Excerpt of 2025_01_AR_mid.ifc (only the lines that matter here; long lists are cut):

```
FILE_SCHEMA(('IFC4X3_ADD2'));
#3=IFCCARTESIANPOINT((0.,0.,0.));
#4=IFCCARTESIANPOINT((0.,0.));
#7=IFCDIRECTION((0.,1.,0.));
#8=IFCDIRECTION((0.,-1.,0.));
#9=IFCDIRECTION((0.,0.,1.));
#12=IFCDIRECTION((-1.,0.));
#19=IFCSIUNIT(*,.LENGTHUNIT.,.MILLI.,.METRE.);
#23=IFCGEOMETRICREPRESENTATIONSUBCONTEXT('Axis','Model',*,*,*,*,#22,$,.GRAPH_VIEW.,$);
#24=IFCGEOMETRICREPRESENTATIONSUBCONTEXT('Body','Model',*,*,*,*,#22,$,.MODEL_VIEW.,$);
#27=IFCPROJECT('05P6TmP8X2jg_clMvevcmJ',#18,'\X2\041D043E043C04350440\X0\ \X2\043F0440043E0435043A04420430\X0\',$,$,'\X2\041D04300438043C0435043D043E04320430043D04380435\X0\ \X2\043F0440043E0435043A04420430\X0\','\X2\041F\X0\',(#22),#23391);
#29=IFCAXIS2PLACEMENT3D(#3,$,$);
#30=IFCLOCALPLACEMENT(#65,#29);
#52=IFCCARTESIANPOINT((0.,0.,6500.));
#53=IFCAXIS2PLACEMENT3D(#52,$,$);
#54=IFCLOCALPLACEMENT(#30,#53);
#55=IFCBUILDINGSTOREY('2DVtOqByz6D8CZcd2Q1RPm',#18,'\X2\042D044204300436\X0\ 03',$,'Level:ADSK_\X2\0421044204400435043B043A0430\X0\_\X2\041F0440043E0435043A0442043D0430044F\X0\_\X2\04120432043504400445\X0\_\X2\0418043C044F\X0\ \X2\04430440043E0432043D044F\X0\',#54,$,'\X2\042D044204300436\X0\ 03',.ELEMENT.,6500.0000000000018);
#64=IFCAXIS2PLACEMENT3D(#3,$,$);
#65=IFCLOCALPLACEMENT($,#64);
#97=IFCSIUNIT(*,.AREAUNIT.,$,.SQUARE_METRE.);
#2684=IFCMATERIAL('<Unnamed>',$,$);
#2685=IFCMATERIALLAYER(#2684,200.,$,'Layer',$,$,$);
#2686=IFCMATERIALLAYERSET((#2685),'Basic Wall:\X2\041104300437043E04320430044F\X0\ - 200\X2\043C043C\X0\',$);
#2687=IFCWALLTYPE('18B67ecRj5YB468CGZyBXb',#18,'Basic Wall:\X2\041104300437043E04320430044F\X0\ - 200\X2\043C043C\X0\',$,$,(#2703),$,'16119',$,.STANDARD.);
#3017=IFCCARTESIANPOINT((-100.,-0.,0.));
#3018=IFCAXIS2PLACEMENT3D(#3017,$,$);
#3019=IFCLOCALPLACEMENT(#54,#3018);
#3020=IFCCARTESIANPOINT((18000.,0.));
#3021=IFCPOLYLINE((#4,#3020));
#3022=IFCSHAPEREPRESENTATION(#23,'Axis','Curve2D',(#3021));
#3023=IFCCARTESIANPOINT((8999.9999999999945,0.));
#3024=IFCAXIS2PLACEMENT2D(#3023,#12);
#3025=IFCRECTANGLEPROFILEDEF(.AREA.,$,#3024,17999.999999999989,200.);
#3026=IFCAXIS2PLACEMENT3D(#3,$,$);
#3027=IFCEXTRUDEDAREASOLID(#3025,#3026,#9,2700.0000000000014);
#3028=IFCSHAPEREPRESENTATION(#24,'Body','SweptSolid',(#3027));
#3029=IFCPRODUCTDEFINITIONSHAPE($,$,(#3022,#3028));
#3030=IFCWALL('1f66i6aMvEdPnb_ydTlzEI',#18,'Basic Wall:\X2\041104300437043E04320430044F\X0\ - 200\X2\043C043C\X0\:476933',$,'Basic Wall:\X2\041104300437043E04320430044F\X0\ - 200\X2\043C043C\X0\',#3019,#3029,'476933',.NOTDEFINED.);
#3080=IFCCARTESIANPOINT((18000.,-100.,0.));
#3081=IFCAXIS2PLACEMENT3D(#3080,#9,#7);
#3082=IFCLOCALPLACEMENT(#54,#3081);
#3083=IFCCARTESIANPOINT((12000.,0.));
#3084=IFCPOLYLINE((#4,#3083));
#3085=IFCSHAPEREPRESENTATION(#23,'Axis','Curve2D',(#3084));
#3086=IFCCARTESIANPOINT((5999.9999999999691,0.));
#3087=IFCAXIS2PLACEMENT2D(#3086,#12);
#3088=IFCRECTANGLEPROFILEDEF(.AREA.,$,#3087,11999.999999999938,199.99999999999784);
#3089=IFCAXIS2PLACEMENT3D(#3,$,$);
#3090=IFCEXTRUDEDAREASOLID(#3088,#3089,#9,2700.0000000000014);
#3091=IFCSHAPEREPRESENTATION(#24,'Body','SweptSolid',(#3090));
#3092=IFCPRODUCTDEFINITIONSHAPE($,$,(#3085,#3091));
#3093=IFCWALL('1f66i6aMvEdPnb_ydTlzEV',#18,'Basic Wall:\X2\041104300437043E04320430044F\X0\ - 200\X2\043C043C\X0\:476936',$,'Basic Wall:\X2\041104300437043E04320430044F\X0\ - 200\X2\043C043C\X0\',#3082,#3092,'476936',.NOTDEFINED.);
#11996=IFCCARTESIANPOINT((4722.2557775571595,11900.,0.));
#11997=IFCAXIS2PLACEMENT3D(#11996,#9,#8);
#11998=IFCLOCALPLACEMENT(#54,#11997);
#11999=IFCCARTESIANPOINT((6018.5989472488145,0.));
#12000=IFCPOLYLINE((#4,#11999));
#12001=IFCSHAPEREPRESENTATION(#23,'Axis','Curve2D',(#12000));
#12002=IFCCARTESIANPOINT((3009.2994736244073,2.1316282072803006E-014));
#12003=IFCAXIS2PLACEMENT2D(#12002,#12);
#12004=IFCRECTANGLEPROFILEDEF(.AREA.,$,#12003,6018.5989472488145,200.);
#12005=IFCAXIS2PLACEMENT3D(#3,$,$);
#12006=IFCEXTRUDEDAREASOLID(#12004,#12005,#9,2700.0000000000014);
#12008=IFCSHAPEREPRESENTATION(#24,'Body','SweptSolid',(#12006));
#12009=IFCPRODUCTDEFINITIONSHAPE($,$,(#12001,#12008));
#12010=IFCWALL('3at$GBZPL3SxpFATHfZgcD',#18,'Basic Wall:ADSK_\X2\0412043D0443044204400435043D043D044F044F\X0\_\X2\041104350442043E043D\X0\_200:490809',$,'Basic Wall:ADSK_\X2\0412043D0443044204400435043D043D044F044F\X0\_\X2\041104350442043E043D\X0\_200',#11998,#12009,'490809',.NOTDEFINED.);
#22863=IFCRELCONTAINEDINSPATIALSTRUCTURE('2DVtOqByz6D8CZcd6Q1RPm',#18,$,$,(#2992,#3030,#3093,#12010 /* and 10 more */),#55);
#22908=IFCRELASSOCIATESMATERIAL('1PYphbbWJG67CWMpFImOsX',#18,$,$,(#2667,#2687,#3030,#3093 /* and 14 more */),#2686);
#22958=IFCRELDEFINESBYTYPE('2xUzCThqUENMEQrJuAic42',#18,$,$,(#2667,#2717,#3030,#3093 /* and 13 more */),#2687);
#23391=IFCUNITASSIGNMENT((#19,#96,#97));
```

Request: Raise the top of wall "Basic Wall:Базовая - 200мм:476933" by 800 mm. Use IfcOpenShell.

```python
import ifcopenshell
import ifcopenshell.geom
import ifcopenshell.util.representation
import ifcopenshell.util.shape
import ifcopenshell.util.unit

model = ifcopenshell.open("2025_01_AR_mid.ifc")
unit_scale = ifcopenshell.util.unit.calculate_unit_scale(model)
settings = ifcopenshell.geom.settings()


def volume(element):
    """Net volume in cubic metres, openings subtracted."""
    shape = ifcopenshell.geom.create_shape(settings, element)
    return ifcopenshell.util.shape.get_volume(shape.geometry)


wall = model.by_guid("1f66i6aMvEdPnb_ydTlzEI")
before = volume(wall)

body = ifcopenshell.util.representation.get_representation(wall, "Model", "Body")
solid = body.Items[0]
old_height = solid.Depth
solid.Depth += 0.8 / unit_scale
after = volume(wall)

print(f"height {old_height:g} -> {solid.Depth:g}, volume {before:.3f} -> {after:.3f} m3")

model.write("2025_01_AR_mid_rev.ifc")
```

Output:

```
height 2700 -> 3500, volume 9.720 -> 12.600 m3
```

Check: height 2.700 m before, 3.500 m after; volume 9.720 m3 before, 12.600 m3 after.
